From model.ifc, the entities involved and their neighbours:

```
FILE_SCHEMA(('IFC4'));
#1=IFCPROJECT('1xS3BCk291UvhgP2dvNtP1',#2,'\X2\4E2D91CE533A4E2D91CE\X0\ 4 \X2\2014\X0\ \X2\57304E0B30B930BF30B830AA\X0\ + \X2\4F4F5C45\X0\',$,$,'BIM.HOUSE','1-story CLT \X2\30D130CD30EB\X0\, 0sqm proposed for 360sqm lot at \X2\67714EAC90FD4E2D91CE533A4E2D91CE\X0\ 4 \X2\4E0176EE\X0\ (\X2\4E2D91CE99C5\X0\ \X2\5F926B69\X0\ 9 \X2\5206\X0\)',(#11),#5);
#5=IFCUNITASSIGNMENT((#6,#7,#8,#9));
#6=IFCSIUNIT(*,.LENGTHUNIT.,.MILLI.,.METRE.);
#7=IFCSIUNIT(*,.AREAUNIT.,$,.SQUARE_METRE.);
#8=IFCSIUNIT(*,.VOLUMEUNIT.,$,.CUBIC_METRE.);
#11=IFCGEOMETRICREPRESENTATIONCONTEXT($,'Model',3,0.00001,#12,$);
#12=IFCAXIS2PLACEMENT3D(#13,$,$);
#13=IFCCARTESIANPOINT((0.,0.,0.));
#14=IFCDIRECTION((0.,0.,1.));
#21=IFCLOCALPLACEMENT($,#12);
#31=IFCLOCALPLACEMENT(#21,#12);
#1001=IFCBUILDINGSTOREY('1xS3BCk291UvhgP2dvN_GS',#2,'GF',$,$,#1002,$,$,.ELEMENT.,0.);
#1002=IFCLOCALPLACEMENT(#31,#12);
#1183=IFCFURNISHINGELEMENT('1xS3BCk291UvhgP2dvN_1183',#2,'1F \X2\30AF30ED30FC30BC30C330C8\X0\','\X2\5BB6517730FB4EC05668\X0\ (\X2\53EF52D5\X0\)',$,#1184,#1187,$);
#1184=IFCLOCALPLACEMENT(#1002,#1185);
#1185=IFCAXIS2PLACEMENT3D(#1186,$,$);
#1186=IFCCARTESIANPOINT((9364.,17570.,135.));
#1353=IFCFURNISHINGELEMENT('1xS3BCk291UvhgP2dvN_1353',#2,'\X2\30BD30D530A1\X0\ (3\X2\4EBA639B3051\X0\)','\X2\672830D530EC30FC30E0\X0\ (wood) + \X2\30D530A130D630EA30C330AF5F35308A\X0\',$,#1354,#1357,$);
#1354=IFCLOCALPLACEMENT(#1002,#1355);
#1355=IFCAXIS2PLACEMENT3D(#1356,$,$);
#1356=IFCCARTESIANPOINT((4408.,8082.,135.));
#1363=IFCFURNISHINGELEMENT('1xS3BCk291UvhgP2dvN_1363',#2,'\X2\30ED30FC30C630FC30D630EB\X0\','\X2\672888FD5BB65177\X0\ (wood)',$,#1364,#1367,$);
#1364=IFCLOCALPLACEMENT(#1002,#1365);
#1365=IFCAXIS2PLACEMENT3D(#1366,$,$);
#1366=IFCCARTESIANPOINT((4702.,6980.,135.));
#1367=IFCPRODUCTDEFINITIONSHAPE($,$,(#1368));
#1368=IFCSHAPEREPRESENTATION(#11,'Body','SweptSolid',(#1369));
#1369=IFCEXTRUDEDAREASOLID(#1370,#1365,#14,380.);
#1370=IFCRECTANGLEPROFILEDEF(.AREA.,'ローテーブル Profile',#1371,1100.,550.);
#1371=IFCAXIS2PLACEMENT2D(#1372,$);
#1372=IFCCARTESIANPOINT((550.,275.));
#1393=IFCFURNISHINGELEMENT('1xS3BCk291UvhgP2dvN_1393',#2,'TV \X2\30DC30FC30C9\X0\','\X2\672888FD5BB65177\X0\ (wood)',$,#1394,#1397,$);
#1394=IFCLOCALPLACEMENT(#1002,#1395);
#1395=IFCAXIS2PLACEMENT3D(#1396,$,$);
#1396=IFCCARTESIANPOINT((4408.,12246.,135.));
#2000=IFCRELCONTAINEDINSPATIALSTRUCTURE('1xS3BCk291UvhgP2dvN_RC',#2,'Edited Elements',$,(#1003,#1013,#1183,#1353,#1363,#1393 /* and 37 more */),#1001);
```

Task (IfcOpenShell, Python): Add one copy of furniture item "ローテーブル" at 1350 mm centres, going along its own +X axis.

```python
import ifcopenshell
import ifcopenshell.api.geometry
import ifcopenshell.api.root
import ifcopenshell.util.element
import ifcopenshell.util.placement

model = ifcopenshell.open("model.ifc")


def reuse_history(source, copy):
    """copy_class also copies each property set's owner history, people and application; keep the originals."""
    for rel in copy.IsDefinedBy:
        if rel.is_a("IfcRelDefinesByProperties") and (history := rel.RelatingPropertyDefinition.OwnerHistory):
            rel.RelatingPropertyDefinition.OwnerHistory = source.OwnerHistory
            ifcopenshell.util.element.remove_deep2(model, history)


source = model.by_guid("1xS3BCk291UvhgP2dvN_1363")
base = ifcopenshell.util.placement.get_local_placement(source.ObjectPlacement)
step = base[:3, 0] * 1350.0

for i in range(1, 2):
    copy = ifcopenshell.api.root.copy_class(model, product=source)
    copy.Representation = ifcopenshell.util.element.copy_deep(
        model, source.Representation, exclude=["IfcGeometricRepresentationContext", "IfcRepresentationMap"]
    )
    reuse_history(source, copy)
    matrix = base.copy()
    matrix[:3, 3] += i * step
    print("added at", matrix[:3, 3].round(3) + 0.0)
    ifcopenshell.api.geometry.edit_object_placement(model, product=copy, matrix=matrix, is_si=False)

model.write("model_rev.ifc")
```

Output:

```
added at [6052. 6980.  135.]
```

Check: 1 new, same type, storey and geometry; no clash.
